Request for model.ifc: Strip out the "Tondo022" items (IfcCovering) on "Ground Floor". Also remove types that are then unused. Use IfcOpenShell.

First a look at what the model holds.

```python
import ifcopenshell
import ifcopenshell.util.element

model = ifcopenshell.open("model.ifc")
print(model.schema)
storey = next(s for s in model.by_type("IfcBuildingStorey") if s.Name == "Ground Floor")
coverings = [e for e in ifcopenshell.util.element.get_decomposition(storey) if e.is_a("IfcCovering")]
seen = {}
for e in coverings:
    element_type = ifcopenshell.util.element.get_type(e)
    name = element_type.Name if element_type not in (None, e) else None
    seen[name] = seen.get(name, 0) + 1
for name, count in sorted(seen.items(), key=str):
    print(count, "x", name)
```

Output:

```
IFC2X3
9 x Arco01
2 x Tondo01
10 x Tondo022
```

```python
import ifcopenshell
import ifcopenshell.api.root
import ifcopenshell.util.element

model = ifcopenshell.open("model.ifc")

storey = next(s for s in model.by_type("IfcBuildingStorey") if s.Name == "Ground Floor")
coverings = [e for e in ifcopenshell.util.element.get_decomposition(storey) if e.is_a("IfcCovering")]
targets = [e for e in coverings if (t := ifcopenshell.util.element.get_type(e)) not in (None, e) and t.Name == "Tondo022"]
types = {ifcopenshell.util.element.get_type(e) for e in targets} - {None, *targets}

for e in targets:
    ifcopenshell.api.root.remove_product(model, product=e)
print(len(targets), "removed")

unused = [t for t in types if not ifcopenshell.util.element.get_types(t)]
for t in unused:
    ifcopenshell.api.root.remove_product(model, product=t)
print(len(unused), "unused types removed")

model.write("model-out.ifc")
```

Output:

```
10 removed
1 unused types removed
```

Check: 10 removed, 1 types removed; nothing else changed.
